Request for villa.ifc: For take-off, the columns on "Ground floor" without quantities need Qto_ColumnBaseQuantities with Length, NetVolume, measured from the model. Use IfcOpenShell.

First a look at what the model holds.

```python
import ifcopenshell
import ifcopenshell.util.element
import ifcopenshell.util.unit

model = ifcopenshell.open("villa.ifc")
print(model.schema)
for unit_type in ("LENGTHUNIT", "AREAUNIT", "VOLUMEUNIT"):
    print(unit_type, ifcopenshell.util.unit.calculate_unit_scale(model, unit_type))
storey = next(s for s in model.by_type("IfcBuildingStorey") if s.Name == "Ground floor")
columns = [e for e in ifcopenshell.util.element.get_decomposition(storey) if e.is_a("IfcColumn")]
for e in sorted(columns, key=lambda e: e.id()):
    print(e.id(), e.is_a(), e.Name, list(ifcopenshell.util.element.get_psets(e, qtos_only=True)), sep=" | ")
```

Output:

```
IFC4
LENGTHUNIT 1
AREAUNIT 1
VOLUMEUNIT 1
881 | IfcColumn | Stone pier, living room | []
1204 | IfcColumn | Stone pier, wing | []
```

```python
import ifcopenshell
import ifcopenshell.api.pset
import ifcopenshell.geom
import ifcopenshell.util.element
import ifcopenshell.util.shape
import ifcopenshell.util.unit

model = ifcopenshell.open("villa.ifc")
unit_scale = ifcopenshell.util.unit.calculate_unit_scale(model)
volume_scale = ifcopenshell.util.unit.calculate_unit_scale(model, "VOLUMEUNIT")
settings = ifcopenshell.geom.settings()

storey = next(s for s in model.by_type("IfcBuildingStorey") if s.Name == "Ground floor")
columns = [e for e in ifcopenshell.util.element.get_decomposition(storey) if e.is_a("IfcColumn")]

for e in sorted(columns, key=lambda e: e.id()):
    if ifcopenshell.util.element.get_psets(e, qtos_only=True, should_inherit=False):
        continue
    # Geometry comes back in metres, in the element's own axes.
    shape = ifcopenshell.geom.create_shape(settings, e)
    values = {
        "Length": ifcopenshell.util.shape.get_z(shape.geometry) / unit_scale,
        "NetVolume": ifcopenshell.util.shape.get_volume(shape.geometry) / volume_scale,
    }
    qto = ifcopenshell.api.pset.add_qto(model, product=e, name="Qto_ColumnBaseQuantities")
    ifcopenshell.api.pset.edit_qto(model, qto=qto, properties=values)
    print(e.id(), {k: round(v, 3) for k, v in values.items()})

model.write("villa-out.ifc")
```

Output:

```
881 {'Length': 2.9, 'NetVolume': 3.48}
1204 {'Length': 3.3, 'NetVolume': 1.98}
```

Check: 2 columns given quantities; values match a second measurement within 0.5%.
